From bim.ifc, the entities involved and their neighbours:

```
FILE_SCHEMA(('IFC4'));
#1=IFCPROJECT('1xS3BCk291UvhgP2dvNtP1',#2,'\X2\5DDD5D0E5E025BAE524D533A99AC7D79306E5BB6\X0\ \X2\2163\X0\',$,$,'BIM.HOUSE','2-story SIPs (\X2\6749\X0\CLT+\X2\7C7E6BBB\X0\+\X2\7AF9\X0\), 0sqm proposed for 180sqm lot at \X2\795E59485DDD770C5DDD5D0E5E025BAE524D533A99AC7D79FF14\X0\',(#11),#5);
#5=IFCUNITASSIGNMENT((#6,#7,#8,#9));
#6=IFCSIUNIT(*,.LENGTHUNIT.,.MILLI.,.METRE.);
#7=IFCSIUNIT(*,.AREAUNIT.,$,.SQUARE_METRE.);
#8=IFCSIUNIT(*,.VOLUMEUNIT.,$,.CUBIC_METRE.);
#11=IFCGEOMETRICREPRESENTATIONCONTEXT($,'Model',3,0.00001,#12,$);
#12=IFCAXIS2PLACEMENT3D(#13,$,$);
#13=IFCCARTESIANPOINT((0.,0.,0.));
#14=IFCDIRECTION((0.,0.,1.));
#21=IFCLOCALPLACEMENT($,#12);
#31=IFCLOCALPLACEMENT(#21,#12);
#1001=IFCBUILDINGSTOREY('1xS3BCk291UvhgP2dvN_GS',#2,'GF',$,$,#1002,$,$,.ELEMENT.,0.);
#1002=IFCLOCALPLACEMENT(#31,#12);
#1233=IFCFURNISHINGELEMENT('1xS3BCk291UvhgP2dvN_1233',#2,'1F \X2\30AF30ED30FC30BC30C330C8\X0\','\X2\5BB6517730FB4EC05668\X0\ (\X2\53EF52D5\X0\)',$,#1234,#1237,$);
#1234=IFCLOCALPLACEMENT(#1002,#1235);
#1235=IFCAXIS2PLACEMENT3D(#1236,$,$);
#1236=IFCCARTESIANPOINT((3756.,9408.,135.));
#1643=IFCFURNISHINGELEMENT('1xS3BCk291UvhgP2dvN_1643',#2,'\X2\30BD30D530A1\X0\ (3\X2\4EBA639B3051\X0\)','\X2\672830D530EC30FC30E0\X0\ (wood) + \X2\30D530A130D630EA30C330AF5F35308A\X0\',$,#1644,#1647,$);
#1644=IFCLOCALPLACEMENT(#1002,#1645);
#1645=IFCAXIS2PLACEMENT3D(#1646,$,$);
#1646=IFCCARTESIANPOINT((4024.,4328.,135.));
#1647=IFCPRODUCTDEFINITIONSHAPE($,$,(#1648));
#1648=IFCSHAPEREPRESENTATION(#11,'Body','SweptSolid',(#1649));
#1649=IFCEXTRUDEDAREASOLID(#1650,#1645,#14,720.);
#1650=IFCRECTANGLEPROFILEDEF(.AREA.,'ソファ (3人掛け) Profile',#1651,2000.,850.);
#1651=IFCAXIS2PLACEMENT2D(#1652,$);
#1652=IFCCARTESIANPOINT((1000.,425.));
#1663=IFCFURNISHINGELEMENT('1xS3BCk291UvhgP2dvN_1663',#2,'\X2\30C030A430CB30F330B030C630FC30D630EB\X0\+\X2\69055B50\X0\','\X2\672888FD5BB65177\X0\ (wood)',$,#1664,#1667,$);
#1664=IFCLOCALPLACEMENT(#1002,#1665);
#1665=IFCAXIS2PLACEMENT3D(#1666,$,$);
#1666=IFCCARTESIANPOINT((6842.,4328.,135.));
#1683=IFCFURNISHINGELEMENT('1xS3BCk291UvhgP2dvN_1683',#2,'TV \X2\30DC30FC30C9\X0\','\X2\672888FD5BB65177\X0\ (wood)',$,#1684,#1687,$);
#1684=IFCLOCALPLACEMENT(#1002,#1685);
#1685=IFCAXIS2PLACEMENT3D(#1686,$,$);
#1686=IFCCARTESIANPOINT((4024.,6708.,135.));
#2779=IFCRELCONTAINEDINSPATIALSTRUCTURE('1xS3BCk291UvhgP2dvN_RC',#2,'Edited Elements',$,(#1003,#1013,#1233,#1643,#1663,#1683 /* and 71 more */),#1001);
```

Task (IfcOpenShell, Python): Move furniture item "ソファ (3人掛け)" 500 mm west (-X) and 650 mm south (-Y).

```python
import ifcopenshell
import ifcopenshell.api.geometry
import ifcopenshell.util.placement
import ifcopenshell.util.unit

model = ifcopenshell.open("bim.ifc")
unit_scale = ifcopenshell.util.unit.calculate_unit_scale(model)

item = model.by_id(1643)
matrix = ifcopenshell.util.placement.get_local_placement(item.ObjectPlacement)
matrix[0, 3] -= 0.5 / unit_scale
matrix[1, 3] -= 0.65 / unit_scale
ifcopenshell.api.geometry.edit_object_placement(model, product=item, matrix=matrix, is_si=False)

print(ifcopenshell.util.placement.get_local_placement(item.ObjectPlacement).round(3) + 0.0)

model.write("bim_updated.ifc")
```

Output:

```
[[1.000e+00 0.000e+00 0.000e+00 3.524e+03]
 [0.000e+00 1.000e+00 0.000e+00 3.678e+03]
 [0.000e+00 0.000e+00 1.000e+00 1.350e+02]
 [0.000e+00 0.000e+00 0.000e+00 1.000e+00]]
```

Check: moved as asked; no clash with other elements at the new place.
